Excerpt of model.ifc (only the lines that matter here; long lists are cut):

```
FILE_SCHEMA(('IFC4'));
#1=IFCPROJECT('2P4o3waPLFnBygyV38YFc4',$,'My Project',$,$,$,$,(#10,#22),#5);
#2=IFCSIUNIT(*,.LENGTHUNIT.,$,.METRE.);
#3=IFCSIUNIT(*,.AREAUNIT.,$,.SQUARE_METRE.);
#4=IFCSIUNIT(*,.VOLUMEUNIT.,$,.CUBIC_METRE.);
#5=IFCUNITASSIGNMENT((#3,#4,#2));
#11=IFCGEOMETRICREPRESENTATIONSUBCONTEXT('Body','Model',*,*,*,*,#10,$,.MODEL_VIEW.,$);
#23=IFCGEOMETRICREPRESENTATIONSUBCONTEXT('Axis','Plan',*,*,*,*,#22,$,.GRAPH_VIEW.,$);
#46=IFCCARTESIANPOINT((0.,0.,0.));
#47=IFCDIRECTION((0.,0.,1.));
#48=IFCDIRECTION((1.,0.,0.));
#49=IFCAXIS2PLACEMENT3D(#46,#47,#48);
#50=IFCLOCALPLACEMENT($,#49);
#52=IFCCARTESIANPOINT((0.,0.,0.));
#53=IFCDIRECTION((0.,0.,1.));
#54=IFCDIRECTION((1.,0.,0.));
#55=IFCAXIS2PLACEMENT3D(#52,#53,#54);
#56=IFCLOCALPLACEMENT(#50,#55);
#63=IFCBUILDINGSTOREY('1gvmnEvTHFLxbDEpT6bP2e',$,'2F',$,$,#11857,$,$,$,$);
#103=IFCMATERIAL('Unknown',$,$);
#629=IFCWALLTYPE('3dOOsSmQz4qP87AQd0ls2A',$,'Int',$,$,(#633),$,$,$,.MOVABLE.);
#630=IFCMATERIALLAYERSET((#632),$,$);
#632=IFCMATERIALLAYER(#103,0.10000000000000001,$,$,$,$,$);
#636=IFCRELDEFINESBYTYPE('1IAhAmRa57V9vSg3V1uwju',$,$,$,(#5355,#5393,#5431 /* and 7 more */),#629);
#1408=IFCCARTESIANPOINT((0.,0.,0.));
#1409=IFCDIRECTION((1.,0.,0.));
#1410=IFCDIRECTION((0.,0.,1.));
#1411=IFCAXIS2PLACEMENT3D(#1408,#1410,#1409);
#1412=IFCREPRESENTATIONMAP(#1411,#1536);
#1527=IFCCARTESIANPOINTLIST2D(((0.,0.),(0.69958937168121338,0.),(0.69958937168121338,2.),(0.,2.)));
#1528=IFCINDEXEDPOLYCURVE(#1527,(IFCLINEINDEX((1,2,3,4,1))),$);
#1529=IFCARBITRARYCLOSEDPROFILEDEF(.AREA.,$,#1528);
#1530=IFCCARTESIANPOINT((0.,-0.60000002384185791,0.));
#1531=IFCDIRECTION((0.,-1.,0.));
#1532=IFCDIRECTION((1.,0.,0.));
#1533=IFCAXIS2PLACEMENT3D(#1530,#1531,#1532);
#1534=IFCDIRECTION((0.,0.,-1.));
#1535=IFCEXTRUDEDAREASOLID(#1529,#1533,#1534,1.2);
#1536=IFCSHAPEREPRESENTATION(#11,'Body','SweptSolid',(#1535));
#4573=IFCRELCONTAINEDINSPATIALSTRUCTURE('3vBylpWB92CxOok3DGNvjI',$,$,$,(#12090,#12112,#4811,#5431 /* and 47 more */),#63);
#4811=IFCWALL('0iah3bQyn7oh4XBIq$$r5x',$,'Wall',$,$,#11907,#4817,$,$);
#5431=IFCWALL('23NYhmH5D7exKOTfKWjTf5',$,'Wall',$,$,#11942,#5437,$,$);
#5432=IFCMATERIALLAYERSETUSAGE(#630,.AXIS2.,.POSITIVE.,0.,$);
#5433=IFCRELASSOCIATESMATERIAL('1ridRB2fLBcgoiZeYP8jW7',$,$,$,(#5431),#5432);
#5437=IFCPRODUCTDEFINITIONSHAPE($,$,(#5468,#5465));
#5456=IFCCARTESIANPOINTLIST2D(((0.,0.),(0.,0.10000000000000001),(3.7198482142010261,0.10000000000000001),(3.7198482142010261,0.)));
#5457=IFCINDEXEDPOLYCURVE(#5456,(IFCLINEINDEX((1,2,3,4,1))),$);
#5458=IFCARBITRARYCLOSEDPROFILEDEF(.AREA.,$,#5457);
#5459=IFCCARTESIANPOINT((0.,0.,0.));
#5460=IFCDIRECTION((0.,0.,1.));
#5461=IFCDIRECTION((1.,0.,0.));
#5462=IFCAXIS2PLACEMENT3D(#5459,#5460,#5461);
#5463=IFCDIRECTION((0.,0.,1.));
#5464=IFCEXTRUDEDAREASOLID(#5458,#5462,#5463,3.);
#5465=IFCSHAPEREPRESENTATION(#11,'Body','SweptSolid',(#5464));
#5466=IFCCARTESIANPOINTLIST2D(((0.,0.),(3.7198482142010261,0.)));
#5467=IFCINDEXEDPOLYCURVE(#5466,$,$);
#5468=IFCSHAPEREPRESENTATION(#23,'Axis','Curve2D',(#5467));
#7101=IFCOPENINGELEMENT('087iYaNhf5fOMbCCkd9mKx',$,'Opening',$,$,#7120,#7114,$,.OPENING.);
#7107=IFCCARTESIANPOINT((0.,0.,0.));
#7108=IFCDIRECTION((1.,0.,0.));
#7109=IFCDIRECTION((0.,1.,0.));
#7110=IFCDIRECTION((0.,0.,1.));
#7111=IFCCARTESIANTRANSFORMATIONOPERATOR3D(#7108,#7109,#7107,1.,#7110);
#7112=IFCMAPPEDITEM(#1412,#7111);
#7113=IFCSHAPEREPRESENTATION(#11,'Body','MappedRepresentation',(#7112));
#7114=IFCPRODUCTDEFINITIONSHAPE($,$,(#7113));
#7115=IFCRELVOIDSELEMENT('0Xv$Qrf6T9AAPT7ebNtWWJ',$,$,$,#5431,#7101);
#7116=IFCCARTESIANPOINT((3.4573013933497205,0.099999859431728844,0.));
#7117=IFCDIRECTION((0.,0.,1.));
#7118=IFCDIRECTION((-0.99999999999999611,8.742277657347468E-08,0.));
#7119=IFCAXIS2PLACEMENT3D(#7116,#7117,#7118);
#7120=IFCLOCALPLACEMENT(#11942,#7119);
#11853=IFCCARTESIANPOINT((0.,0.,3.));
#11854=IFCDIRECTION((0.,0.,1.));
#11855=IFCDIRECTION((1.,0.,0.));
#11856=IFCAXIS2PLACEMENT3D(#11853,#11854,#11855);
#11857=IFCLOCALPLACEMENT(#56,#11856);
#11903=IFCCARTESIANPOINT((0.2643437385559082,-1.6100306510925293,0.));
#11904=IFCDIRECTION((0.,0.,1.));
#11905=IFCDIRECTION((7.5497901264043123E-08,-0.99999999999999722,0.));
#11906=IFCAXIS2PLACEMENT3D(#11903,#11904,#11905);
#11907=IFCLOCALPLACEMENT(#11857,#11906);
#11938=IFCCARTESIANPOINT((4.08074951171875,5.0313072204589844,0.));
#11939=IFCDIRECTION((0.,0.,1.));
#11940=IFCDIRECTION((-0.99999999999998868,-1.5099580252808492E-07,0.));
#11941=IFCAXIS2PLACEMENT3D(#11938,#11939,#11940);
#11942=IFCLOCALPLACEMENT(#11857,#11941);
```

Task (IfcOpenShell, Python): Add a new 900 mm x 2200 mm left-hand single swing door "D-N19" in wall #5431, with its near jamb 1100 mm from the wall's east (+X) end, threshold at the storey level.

```python
import numpy as np
import ifcopenshell
import ifcopenshell.api.feature
import ifcopenshell.api.geometry
import ifcopenshell.api.root
import ifcopenshell.api.spatial
import ifcopenshell.geom
import ifcopenshell.util.element
import ifcopenshell.util.placement
import ifcopenshell.util.representation
import ifcopenshell.util.shape
import ifcopenshell.util.unit

model = ifcopenshell.open("model.ifc")
unit_scale = ifcopenshell.util.unit.calculate_unit_scale(model)
settings = ifcopenshell.geom.settings()


def volume(element):
    """Net volume in cubic metres, openings subtracted."""
    shape = ifcopenshell.geom.create_shape(settings, element)
    return ifcopenshell.util.shape.get_volume(shape.geometry)


wall = model.by_guid("23NYhmH5D7exKOTfKWjTf5")
storey = ifcopenshell.util.element.get_container(wall, ifc_class="IfcBuildingStorey")
context = ifcopenshell.util.representation.get_context(model, "Model", "Body", "MODEL_VIEW")
before = volume(wall)

width, height, from_end, sill = 0.9, 2.2, 1.1, 0.0  # metres

# The wall runs along its own X axis, and the end named is its -X end.
wall_shape = ifcopenshell.geom.create_shape(settings, wall)
x, y, z = ifcopenshell.util.shape.get_vertices(wall_shape.geometry).T
start = x.min() + from_end
face, thickness = float(y.min()), float(y.max() - y.min())
wall_matrix = ifcopenshell.util.placement.get_local_placement(wall.ObjectPlacement)
level = ifcopenshell.util.placement.get_local_placement(storey.ObjectPlacement)[2, 3]


def in_wall(x, y):
    """Placement at x, y metres in the wall's axes, at sill height."""
    matrix = wall_matrix.copy()
    matrix[:, 3] = wall_matrix @ np.array([x / unit_scale, y / unit_scale, 0.0, 1.0])
    matrix[2, 3] = level + sill / unit_scale
    return matrix


# Opening: a box that overshoots both wall faces by 50 mm.
opening = ifcopenshell.api.root.create_entity(model, ifc_class="IfcOpeningElement", predefined_type="OPENING")
box = ifcopenshell.api.geometry.add_wall_representation(
    model, context=context, length=width, height=height, thickness=thickness + 0.1
)
ifcopenshell.api.geometry.assign_representation(model, product=opening, representation=box)
ifcopenshell.api.geometry.edit_object_placement(model, product=opening, matrix=in_wall(start, face - 0.05), is_si=False)
ifcopenshell.api.feature.add_feature(model, feature=opening, element=wall)

door = ifcopenshell.api.root.create_entity(model, ifc_class="IfcDoor", name="D-N19", predefined_type="DOOR")
door.OverallWidth, door.OverallHeight = width / unit_scale, height / unit_scale
door.OperationType = "SINGLE_SWING_LEFT"
body = ifcopenshell.api.geometry.add_door_representation(
    model,
    context=context,
    overall_width=door.OverallWidth,
    overall_height=door.OverallHeight,
    operation_type="SINGLE_SWING_LEFT",
    lining_properties={"LiningDepth": thickness / unit_scale, "ThresholdDepth": thickness / unit_scale},
)
ifcopenshell.api.geometry.assign_representation(model, product=door, representation=body)
ifcopenshell.api.spatial.assign_container(model, products=[door], relating_structure=storey)
ifcopenshell.api.feature.add_filling(model, opening=opening, element=door)

# The lining spans the wall, so the door starts at the wall face.
ifcopenshell.api.geometry.edit_object_placement(model, product=door, matrix=in_wall(start, face), is_si=False)

after = volume(wall)

print(f"wall volume {before:.3f} -> {after:.3f} m3")

model.write("model_v2.ifc")
```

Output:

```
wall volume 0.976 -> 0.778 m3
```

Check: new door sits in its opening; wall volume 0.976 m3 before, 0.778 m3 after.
